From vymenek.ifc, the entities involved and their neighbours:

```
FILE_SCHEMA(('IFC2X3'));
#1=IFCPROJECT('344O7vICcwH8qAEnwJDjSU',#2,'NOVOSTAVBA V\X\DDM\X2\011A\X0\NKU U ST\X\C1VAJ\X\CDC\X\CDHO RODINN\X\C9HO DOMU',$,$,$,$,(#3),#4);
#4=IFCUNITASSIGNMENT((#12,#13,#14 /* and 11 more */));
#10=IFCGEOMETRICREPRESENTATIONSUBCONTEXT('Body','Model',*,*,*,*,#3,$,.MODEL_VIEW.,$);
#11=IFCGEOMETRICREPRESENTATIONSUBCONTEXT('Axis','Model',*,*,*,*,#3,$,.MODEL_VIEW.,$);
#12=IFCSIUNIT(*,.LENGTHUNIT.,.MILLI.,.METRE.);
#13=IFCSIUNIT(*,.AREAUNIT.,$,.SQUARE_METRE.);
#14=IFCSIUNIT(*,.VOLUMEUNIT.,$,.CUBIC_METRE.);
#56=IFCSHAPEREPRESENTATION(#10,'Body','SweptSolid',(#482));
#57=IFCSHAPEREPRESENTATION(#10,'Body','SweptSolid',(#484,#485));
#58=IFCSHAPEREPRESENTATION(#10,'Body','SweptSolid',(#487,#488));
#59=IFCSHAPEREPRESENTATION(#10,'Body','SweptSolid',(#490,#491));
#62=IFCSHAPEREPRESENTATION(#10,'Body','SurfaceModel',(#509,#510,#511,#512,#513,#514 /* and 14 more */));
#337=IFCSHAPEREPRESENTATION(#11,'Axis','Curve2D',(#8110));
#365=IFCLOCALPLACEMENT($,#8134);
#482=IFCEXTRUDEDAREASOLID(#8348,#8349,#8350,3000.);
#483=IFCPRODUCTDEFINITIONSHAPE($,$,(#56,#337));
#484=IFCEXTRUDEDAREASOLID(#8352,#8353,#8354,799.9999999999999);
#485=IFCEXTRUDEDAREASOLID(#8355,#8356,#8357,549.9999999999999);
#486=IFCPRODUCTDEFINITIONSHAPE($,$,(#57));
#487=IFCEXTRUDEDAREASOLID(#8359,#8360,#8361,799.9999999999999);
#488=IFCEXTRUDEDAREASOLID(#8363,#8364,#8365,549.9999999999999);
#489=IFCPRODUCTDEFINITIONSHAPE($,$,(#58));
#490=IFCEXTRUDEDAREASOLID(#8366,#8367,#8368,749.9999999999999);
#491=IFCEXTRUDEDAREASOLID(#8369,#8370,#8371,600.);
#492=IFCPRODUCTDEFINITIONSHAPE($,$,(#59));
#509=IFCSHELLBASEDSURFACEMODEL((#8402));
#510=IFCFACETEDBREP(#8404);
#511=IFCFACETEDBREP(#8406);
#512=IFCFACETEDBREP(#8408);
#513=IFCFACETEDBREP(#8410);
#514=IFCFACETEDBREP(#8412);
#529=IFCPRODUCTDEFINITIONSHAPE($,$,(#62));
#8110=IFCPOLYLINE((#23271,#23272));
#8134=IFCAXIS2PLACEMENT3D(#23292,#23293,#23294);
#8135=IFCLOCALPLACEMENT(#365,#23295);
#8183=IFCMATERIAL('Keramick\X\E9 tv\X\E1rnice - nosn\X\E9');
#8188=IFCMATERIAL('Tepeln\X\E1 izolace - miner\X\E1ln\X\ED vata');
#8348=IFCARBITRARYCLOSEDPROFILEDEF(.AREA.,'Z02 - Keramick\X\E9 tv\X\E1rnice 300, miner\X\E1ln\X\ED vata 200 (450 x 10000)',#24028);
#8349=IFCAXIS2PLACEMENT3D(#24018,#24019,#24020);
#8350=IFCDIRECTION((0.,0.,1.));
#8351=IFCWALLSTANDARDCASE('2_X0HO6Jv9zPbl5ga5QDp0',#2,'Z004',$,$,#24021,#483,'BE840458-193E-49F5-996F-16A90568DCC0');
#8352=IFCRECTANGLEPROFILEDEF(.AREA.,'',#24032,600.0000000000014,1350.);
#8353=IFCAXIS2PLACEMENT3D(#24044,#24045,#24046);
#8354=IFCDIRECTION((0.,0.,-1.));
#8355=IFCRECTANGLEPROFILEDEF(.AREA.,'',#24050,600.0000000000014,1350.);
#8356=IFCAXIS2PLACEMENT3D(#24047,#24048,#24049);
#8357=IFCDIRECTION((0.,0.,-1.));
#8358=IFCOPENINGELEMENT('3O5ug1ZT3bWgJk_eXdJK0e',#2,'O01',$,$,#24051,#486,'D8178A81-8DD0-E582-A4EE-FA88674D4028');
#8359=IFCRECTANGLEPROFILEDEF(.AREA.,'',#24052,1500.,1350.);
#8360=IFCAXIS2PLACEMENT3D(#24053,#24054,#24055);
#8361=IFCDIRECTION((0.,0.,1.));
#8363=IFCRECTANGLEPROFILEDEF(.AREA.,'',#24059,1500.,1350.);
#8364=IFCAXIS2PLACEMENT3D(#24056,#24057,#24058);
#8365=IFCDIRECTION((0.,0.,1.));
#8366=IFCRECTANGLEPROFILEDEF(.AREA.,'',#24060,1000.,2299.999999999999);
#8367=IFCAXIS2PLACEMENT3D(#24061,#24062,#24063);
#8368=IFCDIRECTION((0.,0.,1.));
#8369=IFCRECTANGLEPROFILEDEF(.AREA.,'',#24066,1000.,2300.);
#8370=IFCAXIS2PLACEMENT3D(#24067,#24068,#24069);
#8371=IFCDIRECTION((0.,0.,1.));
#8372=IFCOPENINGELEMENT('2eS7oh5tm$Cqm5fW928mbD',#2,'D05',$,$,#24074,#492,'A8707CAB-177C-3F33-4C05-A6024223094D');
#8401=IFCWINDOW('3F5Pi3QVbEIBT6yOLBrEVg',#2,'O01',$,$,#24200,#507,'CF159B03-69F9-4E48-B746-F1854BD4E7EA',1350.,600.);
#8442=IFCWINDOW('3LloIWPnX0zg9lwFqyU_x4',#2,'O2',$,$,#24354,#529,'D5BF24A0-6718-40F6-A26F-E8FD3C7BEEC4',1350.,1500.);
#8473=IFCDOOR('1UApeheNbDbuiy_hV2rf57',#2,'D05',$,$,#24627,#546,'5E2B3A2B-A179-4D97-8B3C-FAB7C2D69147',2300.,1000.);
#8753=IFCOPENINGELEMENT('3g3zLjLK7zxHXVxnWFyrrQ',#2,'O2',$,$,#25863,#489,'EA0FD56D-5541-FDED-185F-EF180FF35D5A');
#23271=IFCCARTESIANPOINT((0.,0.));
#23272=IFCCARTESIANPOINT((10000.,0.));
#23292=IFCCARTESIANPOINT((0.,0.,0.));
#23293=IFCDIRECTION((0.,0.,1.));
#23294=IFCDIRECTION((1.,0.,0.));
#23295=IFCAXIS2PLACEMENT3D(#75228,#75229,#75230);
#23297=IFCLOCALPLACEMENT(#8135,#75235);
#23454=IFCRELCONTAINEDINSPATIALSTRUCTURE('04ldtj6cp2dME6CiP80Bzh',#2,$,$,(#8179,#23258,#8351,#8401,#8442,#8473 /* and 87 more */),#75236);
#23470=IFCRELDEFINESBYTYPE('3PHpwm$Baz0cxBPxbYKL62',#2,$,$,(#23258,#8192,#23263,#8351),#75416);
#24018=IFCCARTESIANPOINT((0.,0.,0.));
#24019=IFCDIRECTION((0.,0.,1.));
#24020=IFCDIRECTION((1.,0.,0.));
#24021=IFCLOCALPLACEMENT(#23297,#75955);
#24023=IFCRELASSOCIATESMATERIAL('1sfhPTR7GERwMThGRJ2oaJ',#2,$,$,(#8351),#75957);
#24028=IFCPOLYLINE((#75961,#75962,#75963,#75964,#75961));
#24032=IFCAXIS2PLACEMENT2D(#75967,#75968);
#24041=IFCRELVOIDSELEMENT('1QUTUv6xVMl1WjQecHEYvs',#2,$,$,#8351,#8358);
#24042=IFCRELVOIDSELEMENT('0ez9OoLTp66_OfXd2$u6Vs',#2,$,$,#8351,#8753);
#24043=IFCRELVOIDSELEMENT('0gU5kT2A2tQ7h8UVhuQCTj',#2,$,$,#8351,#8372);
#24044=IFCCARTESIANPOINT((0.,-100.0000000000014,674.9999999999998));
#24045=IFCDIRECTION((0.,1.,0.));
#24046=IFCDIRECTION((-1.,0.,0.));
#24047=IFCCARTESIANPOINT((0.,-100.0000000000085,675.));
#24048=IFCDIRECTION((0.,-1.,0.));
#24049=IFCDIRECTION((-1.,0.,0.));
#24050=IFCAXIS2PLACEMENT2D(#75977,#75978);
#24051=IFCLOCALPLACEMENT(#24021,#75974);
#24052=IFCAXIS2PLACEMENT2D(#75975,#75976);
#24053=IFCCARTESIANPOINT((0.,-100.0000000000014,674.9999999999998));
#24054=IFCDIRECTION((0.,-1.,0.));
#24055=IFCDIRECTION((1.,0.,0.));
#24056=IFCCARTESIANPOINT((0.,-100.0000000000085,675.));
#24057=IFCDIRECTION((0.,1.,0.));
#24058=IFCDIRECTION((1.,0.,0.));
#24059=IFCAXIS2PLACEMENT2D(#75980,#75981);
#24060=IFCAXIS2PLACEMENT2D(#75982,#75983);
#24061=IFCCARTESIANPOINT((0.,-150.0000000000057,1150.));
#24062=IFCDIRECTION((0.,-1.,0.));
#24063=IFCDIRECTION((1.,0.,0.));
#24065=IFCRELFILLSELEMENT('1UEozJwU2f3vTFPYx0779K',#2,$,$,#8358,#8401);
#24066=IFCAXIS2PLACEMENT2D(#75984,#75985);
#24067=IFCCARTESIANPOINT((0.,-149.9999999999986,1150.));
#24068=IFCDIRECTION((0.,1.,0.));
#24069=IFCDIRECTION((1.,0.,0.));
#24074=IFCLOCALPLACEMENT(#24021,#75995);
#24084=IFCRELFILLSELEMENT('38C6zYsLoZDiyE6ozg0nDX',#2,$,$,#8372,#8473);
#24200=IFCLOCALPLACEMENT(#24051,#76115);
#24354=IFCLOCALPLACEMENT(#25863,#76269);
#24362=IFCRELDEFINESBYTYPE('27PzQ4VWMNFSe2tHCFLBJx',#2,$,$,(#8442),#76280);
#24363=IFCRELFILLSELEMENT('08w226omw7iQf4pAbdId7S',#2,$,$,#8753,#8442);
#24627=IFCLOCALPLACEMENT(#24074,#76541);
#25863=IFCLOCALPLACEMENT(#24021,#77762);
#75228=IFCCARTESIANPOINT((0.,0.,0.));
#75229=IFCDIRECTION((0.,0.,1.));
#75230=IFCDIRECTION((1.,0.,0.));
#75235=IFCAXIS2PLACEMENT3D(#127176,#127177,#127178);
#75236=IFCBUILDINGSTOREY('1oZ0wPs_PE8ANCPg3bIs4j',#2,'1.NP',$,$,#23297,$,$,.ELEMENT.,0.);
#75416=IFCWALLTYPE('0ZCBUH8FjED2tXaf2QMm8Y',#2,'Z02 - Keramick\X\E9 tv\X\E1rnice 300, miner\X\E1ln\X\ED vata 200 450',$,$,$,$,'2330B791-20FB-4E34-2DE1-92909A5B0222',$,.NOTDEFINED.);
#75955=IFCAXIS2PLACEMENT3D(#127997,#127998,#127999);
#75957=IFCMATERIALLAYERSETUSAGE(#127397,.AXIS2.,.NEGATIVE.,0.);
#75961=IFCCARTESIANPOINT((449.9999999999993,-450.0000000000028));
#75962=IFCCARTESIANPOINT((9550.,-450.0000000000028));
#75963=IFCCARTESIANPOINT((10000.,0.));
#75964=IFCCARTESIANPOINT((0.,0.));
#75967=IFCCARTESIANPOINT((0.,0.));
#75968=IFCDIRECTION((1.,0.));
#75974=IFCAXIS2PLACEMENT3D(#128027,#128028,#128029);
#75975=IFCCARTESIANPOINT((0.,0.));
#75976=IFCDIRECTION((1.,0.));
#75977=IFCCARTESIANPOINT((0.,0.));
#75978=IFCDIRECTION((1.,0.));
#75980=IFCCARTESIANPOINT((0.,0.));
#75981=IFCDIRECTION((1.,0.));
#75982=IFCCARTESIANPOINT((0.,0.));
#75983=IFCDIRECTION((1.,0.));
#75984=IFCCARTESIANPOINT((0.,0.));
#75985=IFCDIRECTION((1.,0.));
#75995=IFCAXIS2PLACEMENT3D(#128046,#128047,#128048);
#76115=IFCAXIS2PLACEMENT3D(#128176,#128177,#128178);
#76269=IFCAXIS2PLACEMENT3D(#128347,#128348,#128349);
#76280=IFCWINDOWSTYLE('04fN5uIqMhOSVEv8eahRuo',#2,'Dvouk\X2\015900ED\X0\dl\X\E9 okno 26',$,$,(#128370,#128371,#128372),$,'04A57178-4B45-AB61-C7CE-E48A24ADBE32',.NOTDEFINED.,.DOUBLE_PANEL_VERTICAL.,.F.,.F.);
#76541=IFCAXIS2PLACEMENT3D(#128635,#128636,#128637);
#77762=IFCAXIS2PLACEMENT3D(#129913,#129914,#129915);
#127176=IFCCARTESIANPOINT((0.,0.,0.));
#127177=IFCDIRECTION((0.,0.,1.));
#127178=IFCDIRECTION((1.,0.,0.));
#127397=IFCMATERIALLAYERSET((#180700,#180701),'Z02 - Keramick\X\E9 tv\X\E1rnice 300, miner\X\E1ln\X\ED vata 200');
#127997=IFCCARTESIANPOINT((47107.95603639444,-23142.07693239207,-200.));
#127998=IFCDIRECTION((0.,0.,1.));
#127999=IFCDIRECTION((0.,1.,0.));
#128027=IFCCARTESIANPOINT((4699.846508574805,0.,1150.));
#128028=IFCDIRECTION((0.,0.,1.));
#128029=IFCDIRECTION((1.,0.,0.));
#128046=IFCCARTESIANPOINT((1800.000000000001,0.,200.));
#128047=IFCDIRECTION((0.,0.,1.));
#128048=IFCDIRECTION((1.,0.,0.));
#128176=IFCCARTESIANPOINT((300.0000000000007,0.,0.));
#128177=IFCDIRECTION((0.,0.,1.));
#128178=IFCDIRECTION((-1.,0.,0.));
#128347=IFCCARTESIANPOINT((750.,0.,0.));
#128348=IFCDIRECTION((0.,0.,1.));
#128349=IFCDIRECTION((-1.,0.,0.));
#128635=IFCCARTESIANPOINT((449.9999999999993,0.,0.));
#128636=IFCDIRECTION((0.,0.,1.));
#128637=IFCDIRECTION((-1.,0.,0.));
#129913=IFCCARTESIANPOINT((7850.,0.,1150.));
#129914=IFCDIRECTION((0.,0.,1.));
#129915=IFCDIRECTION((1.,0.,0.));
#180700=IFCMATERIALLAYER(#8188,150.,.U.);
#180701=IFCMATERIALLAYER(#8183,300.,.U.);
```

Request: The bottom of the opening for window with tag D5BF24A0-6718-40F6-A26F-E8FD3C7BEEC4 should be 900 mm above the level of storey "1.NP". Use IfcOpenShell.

```python
import numpy as np
import ifcopenshell
import ifcopenshell.api.geometry
import ifcopenshell.geom
import ifcopenshell.util.element
import ifcopenshell.util.placement
import ifcopenshell.util.shape
import ifcopenshell.util.unit

model = ifcopenshell.open("vymenek.ifc")
unit_scale = ifcopenshell.util.unit.calculate_unit_scale(model)

window = model.by_id(8442)
opening = window.FillsVoids[0].RelatingOpeningElement
storey = ifcopenshell.util.element.get_container(window, ifc_class="IfcBuildingStorey")
level = ifcopenshell.util.placement.get_local_placement(storey.ObjectPlacement)[2, 3]

# The opening's origin need not be at the sill, so measure its lowest point.
shape = ifcopenshell.geom.create_shape(ifcopenshell.geom.settings(), opening)
bottom = ifcopenshell.util.shape.get_shape_bottom_elevation(shape, shape.geometry) / unit_scale
dz = level + 0.9 / unit_scale - bottom

shift = np.array([0.0, 0.0, dz])
# The window is placed relative to its opening, so it follows when the opening moves.
matrix = ifcopenshell.util.placement.get_local_placement(opening.ObjectPlacement)
matrix[:3, 3] += shift
ifcopenshell.api.geometry.edit_object_placement(
    model, product=opening, matrix=matrix, is_si=False, should_transform_children=True
)

print(f"moved by {dz * unit_scale:+.3f} m")

model.write("vymenek_v2.ifc")
```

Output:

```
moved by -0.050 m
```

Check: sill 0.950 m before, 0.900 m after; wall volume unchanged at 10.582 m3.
